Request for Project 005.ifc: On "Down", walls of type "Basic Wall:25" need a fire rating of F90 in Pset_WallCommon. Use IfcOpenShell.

First a look at what the model holds.

```python
import ifcopenshell
import ifcopenshell.util.element

model = ifcopenshell.open("Project 005.ifc")
print(model.schema)
storey = next(s for s in model.by_type("IfcBuildingStorey") if s.Name == "Down")
walls = [e for e in ifcopenshell.util.element.get_decomposition(storey) if e.is_a("IfcWall")]
seen = {}
for e in walls:
    element_type = ifcopenshell.util.element.get_type(e)
    key = (element_type.Name if element_type != e and element_type else None, ifcopenshell.util.element.get_pset(e, "Pset_WallCommon", "FireRating"))
    seen[key] = seen.get(key, 0) + 1
for (name, value), count in sorted(seen.items(), key=str):
    print(count, "x", name, "|", value)
```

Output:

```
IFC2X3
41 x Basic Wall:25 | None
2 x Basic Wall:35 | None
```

```python
import ifcopenshell
import ifcopenshell.api.pset
import ifcopenshell.util.element

model = ifcopenshell.open("Project 005.ifc")

storey = next(s for s in model.by_type("IfcBuildingStorey") if s.Name == "Down")
walls = [e for e in ifcopenshell.util.element.get_decomposition(storey) if e.is_a("IfcWall")]

count = 0
for e in walls:
    element_type = ifcopenshell.util.element.get_type(e)
    if element_type in (None, e) or element_type.Name != "Basic Wall:25":
        continue
    # add_pset returns the element's existing set when there is one.
    pset = ifcopenshell.api.pset.add_pset(model, product=e, name="Pset_WallCommon")
    ifcopenshell.api.pset.edit_pset(model, pset=pset, properties={"FireRating": "F90"})
    count += 1

print(count, "walls updated")

model.write("Project 005_edited.ifc")
```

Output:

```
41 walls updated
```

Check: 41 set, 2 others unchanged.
